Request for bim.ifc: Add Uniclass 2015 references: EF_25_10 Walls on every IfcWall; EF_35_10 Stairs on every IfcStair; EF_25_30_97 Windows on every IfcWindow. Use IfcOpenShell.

First a look at what the model holds.

```python
import ifcopenshell

model = ifcopenshell.open("bim.ifc")
print(model.schema)
print("classifications:", [c.Name for c in model.by_type("IfcClassification")])
for ifc_class in ("IfcDoor", "IfcRoof", "IfcStair", "IfcWall", "IfcWindow"):
    print(ifc_class, len(model.by_type(ifc_class)))
```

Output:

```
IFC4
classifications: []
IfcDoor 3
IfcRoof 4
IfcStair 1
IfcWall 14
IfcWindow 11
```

```python
import ifcopenshell
import ifcopenshell.api.classification

model = ifcopenshell.open("bim.ifc")

system = ifcopenshell.api.classification.add_classification(model, classification="Uniclass 2015")

codes = {
    "IfcWall": ("EF_25_10", "Walls"),
    "IfcStair": ("EF_35_10", "Stairs"),
    "IfcWindow": ("EF_25_30_97", "Windows"),
}
for ifc_class, (code, name) in codes.items():
    products = model.by_type(ifc_class)
    ifcopenshell.api.classification.add_reference(
        model, products=products, classification=system, identification=code, name=name
    )
    print(code, len(products))

model.write("bim_edited.ifc")
```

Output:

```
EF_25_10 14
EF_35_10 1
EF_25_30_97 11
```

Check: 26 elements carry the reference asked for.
